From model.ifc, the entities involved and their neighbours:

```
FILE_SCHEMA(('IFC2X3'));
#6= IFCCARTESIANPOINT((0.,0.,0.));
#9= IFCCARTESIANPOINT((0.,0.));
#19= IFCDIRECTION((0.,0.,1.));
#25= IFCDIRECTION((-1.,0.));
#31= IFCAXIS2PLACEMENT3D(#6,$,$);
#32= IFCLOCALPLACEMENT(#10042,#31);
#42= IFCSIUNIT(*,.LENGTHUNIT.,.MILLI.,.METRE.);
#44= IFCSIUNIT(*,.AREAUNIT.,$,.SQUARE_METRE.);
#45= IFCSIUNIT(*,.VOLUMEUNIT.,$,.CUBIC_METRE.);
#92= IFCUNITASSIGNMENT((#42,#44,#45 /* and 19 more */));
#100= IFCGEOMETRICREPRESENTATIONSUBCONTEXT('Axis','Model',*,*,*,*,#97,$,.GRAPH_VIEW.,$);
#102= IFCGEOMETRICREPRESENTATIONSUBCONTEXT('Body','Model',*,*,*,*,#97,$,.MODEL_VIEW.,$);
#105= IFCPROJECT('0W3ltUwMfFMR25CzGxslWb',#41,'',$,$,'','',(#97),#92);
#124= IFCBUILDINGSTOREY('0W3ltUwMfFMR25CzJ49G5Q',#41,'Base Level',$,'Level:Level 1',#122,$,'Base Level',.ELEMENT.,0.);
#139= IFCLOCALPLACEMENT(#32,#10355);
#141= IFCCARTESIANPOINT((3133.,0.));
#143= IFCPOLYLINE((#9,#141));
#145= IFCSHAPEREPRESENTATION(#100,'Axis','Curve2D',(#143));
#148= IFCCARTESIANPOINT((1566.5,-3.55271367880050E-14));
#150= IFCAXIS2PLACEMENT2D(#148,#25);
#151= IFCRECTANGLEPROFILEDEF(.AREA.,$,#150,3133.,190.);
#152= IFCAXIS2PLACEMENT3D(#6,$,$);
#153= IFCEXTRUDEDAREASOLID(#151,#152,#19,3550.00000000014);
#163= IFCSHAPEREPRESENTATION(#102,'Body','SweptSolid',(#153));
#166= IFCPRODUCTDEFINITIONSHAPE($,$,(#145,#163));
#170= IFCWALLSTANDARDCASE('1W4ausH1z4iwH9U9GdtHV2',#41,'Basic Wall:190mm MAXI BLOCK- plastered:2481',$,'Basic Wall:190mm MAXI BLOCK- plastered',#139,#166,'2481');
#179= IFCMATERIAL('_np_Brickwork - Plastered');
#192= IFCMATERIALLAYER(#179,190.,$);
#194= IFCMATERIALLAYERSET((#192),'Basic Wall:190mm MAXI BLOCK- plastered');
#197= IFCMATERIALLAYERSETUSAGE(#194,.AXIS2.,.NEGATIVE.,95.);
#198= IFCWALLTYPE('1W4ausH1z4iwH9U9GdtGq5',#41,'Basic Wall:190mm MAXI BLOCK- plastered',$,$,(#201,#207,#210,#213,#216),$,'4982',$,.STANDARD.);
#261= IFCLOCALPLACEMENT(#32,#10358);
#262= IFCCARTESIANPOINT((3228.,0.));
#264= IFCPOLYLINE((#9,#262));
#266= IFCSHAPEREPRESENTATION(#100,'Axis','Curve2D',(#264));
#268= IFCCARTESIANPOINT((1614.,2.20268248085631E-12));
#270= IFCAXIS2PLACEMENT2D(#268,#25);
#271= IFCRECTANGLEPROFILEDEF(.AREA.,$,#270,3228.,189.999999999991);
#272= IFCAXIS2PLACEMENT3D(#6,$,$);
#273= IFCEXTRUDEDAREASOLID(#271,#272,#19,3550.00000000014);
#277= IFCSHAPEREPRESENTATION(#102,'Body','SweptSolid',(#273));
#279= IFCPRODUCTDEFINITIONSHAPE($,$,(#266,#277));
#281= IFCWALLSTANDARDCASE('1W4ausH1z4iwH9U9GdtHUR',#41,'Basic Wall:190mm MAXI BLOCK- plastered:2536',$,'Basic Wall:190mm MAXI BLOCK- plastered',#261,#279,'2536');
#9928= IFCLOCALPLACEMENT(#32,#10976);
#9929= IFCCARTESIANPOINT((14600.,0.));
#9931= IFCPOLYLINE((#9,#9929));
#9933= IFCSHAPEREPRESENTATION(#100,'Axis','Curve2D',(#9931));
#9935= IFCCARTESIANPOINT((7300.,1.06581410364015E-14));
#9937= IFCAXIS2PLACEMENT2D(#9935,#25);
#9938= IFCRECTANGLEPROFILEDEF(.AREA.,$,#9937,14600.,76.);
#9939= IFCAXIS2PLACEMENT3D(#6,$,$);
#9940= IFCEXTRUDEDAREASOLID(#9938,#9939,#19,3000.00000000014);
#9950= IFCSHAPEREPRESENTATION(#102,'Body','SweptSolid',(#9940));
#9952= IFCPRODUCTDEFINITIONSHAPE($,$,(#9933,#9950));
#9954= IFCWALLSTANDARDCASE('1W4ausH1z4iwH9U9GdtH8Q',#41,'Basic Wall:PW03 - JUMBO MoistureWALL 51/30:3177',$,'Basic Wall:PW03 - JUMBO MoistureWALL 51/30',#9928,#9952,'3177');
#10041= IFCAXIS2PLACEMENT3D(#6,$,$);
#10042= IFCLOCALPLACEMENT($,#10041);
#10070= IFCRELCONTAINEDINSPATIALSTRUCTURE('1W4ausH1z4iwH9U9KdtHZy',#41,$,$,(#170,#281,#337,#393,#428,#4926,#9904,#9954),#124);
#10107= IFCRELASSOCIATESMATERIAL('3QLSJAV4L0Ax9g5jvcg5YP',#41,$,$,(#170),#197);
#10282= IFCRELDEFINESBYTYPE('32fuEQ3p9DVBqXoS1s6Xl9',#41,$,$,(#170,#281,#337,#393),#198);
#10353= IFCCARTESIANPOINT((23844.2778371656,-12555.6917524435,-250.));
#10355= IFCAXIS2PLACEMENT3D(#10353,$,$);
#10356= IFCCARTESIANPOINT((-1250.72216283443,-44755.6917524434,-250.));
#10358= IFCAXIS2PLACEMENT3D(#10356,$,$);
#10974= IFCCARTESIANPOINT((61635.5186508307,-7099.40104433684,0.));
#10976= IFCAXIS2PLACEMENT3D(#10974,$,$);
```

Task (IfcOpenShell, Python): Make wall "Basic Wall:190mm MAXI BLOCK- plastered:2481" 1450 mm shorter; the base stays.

```python
import ifcopenshell
import ifcopenshell.geom
import ifcopenshell.util.representation
import ifcopenshell.util.shape
import ifcopenshell.util.unit

model = ifcopenshell.open("model.ifc")
unit_scale = ifcopenshell.util.unit.calculate_unit_scale(model)
settings = ifcopenshell.geom.settings()


def volume(element):
    """Net volume in cubic metres, openings subtracted."""
    shape = ifcopenshell.geom.create_shape(settings, element)
    return ifcopenshell.util.shape.get_volume(shape.geometry)


wall = model.by_id(170)
before = volume(wall)

body = ifcopenshell.util.representation.get_representation(wall, "Model", "Body")
solid = body.Items[0]
old_height = solid.Depth
solid.Depth -= 1.45 / unit_scale
after = volume(wall)

print(f"height {old_height:g} -> {solid.Depth:g}, volume {before:.3f} -> {after:.3f} m3")

model.write("model-out.ifc")
```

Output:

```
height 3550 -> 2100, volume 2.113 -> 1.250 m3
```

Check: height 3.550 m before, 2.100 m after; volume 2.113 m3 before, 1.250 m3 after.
